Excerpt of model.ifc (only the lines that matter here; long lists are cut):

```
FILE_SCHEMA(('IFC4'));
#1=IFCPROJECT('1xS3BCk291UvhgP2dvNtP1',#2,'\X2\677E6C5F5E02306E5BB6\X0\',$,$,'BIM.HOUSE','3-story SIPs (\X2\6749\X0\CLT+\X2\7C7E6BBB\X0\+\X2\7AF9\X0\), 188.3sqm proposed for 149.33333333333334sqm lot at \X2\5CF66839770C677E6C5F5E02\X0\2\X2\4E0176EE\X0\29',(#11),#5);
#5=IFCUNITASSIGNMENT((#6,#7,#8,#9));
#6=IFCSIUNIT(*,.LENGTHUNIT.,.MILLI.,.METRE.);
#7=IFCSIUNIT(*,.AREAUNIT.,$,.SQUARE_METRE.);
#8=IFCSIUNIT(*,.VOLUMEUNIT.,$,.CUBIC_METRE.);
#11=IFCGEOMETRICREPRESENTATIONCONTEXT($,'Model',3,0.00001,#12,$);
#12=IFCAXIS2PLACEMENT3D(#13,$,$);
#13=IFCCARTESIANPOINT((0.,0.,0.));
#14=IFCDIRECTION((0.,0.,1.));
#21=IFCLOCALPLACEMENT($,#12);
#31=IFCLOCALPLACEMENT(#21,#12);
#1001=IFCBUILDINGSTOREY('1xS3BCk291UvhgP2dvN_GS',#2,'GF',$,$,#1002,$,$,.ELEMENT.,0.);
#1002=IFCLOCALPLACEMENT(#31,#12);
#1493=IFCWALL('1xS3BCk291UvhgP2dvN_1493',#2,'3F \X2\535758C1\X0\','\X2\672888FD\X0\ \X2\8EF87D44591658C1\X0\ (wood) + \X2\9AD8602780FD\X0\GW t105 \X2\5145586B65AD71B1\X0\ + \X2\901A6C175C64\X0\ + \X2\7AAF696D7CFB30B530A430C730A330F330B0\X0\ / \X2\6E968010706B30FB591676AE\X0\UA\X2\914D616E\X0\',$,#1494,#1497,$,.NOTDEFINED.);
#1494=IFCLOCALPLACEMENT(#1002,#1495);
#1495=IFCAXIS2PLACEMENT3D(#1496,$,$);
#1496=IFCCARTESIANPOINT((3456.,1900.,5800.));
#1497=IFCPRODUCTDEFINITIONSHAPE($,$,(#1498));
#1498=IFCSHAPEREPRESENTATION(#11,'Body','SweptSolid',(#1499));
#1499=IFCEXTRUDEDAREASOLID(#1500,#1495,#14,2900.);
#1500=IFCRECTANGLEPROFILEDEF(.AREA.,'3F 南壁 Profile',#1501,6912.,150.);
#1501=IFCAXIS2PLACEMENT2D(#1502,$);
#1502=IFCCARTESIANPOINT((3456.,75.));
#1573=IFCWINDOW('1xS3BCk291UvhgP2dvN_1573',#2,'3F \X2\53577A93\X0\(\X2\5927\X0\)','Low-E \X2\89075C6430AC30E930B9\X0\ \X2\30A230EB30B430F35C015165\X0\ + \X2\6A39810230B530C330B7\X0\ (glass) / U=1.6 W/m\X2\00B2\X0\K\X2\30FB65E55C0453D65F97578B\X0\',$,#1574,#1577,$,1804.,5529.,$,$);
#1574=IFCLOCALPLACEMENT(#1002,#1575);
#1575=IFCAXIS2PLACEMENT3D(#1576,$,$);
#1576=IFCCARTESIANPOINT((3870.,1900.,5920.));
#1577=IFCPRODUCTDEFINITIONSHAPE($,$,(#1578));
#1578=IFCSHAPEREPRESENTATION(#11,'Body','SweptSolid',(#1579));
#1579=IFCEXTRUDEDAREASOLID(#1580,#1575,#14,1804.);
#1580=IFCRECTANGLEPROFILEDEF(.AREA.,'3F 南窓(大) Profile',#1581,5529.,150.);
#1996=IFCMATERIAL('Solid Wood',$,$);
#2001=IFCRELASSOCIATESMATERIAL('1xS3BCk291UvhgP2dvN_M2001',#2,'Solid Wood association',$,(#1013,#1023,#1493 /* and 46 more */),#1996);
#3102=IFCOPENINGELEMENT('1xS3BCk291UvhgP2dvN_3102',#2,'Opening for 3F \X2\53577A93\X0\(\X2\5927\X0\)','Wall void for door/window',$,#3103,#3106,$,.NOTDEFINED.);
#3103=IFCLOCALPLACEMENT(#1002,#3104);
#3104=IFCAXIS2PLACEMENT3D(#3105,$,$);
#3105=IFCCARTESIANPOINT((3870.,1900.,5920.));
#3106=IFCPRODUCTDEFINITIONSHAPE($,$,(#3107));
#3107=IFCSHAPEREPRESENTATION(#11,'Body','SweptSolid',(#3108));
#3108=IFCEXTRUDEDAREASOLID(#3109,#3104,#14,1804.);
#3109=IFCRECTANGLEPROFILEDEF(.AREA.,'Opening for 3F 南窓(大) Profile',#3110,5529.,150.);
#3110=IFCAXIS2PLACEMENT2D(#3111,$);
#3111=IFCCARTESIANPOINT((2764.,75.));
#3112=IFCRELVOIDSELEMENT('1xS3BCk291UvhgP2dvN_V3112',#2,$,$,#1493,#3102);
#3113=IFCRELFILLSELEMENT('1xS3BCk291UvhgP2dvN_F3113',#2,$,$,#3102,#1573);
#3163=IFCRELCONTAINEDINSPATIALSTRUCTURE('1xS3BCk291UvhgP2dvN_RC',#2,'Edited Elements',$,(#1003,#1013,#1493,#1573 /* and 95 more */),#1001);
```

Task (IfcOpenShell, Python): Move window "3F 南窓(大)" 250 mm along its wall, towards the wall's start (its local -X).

```python
import ifcopenshell
import ifcopenshell.api.geometry
import ifcopenshell.util.placement
import ifcopenshell.util.unit

model = ifcopenshell.open("model.ifc")
unit_scale = ifcopenshell.util.unit.calculate_unit_scale(model)

window = model.by_guid("1xS3BCk291UvhgP2dvN_1573")
opening = window.FillsVoids[0].RelatingOpeningElement
wall = opening.VoidsElements[0].RelatingBuildingElement

wall_matrix = ifcopenshell.util.placement.get_local_placement(wall.ObjectPlacement)
shift = wall_matrix[:3, 0] * -0.25 / unit_scale
before = ifcopenshell.util.placement.get_local_placement(window.ObjectPlacement)[:3, 3].copy()

# The window is not placed relative to its opening, so move both.
for product in (opening, window):
    matrix = ifcopenshell.util.placement.get_local_placement(product.ObjectPlacement)
    matrix[:3, 3] += shift
    ifcopenshell.api.geometry.edit_object_placement(model, product=product, matrix=matrix, is_si=False)

after = ifcopenshell.util.placement.get_local_placement(window.ObjectPlacement)[:3, 3]
print("window moved by", (after - before).round(3) + 0.0)

model.write("model_rev.ifc")
```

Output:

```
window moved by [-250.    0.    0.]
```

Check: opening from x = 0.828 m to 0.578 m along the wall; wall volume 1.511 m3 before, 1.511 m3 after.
